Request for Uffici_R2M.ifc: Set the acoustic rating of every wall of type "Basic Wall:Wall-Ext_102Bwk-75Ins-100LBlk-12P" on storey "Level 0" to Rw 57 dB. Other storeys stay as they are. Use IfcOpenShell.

First a look at what the model holds.

```python
import ifcopenshell
import ifcopenshell.util.element

model = ifcopenshell.open("Uffici_R2M.ifc")
print(model.schema)
storey = next(s for s in model.by_type("IfcBuildingStorey") if s.Name == "Level 0")
walls = [e for e in ifcopenshell.util.element.get_decomposition(storey) if e.is_a("IfcWall")]
seen = {}
for e in walls:
    element_type = ifcopenshell.util.element.get_type(e)
    key = (element_type.Name if element_type != e and element_type else None, ifcopenshell.util.element.get_pset(e, "Pset_WallCommon", "AcousticRating"))
    seen[key] = seen.get(key, 0) + 1
for (name, value), count in sorted(seen.items(), key=str):
    print(count, "x", name, "|", value)
```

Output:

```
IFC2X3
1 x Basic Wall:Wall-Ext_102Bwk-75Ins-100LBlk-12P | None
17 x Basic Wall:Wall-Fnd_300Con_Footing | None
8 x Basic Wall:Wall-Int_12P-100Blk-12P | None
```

```python
import ifcopenshell
import ifcopenshell.api.pset
import ifcopenshell.util.element

model = ifcopenshell.open("Uffici_R2M.ifc")

storey = next(s for s in model.by_type("IfcBuildingStorey") if s.Name == "Level 0")
walls = [e for e in ifcopenshell.util.element.get_decomposition(storey) if e.is_a("IfcWall")]

count = 0
for e in walls:
    element_type = ifcopenshell.util.element.get_type(e)
    if element_type in (None, e) or element_type.Name != "Basic Wall:Wall-Ext_102Bwk-75Ins-100LBlk-12P":
        continue
    # add_pset returns the element's existing set when there is one.
    pset = ifcopenshell.api.pset.add_pset(model, product=e, name="Pset_WallCommon")
    ifcopenshell.api.pset.edit_pset(model, pset=pset, properties={"AcousticRating": "Rw 57 dB"})
    count += 1

print(count, "walls updated")

model.write("Uffici_R2M_rev.ifc")
```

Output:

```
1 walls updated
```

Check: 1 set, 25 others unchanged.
